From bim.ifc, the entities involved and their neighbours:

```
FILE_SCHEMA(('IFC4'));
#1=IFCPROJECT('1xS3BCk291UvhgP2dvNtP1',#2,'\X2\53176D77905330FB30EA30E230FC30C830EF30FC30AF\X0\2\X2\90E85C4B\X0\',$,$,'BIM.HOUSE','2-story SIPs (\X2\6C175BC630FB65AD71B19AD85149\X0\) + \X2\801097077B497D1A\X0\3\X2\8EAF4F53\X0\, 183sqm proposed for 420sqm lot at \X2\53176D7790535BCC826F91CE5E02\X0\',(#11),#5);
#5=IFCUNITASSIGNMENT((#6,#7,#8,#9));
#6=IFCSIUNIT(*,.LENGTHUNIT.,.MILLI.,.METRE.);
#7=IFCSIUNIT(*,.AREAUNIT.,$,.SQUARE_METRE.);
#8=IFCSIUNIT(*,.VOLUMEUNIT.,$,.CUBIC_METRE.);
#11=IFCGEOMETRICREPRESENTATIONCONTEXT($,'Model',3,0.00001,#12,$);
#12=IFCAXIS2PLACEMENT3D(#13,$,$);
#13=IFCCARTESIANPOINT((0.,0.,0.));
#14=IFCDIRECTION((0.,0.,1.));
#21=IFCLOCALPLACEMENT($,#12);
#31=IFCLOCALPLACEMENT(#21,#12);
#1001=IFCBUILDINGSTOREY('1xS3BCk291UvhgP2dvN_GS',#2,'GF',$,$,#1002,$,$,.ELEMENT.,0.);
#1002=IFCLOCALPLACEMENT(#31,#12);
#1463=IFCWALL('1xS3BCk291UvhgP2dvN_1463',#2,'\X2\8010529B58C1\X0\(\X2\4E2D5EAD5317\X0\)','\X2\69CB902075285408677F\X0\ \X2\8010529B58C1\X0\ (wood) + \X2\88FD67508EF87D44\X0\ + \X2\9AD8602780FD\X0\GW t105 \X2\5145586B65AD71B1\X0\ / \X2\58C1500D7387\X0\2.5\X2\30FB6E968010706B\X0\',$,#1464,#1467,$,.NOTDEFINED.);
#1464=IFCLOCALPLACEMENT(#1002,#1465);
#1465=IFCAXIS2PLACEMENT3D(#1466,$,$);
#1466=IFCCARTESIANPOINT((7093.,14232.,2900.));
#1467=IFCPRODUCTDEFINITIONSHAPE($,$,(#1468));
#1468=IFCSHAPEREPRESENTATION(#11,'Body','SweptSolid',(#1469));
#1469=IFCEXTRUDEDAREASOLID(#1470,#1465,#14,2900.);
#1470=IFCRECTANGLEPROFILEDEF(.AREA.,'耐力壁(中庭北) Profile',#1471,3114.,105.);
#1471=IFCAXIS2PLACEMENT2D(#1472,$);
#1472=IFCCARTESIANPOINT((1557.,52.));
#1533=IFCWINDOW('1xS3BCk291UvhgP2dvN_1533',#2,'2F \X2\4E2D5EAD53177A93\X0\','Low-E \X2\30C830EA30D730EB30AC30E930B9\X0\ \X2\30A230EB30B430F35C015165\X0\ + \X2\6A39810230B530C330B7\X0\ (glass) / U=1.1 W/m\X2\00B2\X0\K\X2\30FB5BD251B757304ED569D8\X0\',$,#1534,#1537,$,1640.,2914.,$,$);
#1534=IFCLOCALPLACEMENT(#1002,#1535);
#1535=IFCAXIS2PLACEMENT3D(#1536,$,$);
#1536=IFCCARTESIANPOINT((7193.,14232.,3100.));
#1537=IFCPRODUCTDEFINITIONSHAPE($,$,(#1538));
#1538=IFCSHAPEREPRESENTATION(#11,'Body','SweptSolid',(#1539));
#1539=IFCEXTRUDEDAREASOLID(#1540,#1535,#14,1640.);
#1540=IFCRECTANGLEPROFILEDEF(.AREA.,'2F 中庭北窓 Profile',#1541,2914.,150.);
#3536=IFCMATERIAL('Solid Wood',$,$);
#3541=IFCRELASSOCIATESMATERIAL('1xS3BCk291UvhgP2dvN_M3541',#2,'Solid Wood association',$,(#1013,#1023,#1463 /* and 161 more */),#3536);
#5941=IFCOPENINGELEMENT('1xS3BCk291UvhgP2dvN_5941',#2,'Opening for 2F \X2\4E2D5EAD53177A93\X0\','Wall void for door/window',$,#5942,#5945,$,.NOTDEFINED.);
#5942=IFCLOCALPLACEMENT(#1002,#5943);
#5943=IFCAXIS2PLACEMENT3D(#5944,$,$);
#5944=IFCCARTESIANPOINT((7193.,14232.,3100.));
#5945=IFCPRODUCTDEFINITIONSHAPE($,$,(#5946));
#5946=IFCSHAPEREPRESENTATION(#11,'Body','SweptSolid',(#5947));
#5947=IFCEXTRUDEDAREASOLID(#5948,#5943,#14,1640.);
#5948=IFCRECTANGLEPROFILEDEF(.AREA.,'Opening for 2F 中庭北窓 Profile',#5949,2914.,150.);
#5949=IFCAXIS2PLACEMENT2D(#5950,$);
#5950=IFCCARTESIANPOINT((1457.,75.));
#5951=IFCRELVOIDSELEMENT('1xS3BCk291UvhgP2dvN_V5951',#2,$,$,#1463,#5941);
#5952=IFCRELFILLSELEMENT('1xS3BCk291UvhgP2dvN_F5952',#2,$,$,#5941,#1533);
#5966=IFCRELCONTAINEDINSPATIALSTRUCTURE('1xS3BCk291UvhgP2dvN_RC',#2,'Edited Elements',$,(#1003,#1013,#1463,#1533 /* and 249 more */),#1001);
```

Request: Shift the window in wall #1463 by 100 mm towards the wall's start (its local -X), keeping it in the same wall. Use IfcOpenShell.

```python
import ifcopenshell
import ifcopenshell.api.geometry
import ifcopenshell.util.placement
import ifcopenshell.util.unit

model = ifcopenshell.open("bim.ifc")
unit_scale = ifcopenshell.util.unit.calculate_unit_scale(model)

window = model.by_guid("1xS3BCk291UvhgP2dvN_1533")
opening = window.FillsVoids[0].RelatingOpeningElement
wall = opening.VoidsElements[0].RelatingBuildingElement

wall_matrix = ifcopenshell.util.placement.get_local_placement(wall.ObjectPlacement)
shift = wall_matrix[:3, 0] * -0.1 / unit_scale
before = ifcopenshell.util.placement.get_local_placement(window.ObjectPlacement)[:3, 3].copy()

# The window is not placed relative to its opening, so move both.
for product in (opening, window):
    matrix = ifcopenshell.util.placement.get_local_placement(product.ObjectPlacement)
    matrix[:3, 3] += shift
    ifcopenshell.api.geometry.edit_object_placement(model, product=product, matrix=matrix, is_si=False)

after = ifcopenshell.util.placement.get_local_placement(window.ObjectPlacement)[:3, 3]
print("window moved by", (after - before).round(3) + 0.0)

model.write("bim_v2.ifc")
```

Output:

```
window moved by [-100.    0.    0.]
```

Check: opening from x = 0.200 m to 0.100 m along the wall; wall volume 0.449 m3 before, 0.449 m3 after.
